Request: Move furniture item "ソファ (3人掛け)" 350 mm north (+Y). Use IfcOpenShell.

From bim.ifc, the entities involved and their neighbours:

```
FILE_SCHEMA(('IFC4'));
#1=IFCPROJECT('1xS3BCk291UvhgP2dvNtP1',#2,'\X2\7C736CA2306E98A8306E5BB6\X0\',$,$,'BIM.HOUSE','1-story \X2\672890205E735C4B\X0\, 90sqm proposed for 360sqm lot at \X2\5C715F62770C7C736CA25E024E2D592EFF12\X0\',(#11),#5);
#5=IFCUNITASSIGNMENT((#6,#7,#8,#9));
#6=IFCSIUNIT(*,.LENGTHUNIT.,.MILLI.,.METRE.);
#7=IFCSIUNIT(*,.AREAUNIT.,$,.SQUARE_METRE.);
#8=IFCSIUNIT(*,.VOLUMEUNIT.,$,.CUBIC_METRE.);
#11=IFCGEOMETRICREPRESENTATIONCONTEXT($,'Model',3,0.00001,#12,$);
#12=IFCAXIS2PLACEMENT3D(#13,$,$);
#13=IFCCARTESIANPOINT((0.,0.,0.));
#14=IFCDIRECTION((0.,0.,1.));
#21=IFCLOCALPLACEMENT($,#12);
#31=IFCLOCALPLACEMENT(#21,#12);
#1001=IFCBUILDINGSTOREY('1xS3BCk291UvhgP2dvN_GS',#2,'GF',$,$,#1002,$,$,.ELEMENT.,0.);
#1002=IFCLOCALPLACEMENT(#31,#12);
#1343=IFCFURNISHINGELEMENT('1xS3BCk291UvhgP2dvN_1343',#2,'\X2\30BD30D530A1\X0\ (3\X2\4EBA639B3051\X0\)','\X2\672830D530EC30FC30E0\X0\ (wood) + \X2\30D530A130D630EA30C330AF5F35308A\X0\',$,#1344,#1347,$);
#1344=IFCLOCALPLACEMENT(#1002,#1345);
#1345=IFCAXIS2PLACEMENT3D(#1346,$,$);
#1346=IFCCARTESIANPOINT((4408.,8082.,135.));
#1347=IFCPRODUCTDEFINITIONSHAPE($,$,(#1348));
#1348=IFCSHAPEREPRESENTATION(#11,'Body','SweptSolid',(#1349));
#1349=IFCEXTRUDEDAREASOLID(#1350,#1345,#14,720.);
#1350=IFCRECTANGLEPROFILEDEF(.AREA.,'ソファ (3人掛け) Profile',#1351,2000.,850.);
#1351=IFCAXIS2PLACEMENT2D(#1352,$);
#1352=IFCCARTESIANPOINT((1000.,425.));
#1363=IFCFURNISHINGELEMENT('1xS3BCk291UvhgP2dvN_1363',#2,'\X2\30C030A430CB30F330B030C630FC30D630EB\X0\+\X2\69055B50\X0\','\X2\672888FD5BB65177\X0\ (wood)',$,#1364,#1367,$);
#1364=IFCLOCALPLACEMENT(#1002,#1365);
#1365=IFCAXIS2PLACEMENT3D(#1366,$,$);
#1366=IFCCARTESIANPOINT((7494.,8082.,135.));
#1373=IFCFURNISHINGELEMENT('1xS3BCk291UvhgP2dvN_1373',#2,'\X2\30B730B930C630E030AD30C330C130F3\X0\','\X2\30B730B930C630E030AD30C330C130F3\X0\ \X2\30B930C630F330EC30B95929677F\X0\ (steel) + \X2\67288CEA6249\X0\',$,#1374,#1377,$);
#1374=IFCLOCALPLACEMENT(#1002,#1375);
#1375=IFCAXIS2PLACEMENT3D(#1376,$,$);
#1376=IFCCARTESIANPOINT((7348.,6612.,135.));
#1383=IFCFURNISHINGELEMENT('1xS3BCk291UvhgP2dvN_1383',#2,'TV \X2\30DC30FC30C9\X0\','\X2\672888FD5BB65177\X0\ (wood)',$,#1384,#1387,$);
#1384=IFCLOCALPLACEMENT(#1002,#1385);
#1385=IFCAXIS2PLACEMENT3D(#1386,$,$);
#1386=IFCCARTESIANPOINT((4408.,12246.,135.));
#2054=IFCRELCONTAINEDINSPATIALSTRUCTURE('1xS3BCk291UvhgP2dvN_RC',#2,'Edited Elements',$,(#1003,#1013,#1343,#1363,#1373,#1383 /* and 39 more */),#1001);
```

```python
import ifcopenshell
import ifcopenshell.api.geometry
import ifcopenshell.util.placement
import ifcopenshell.util.unit

model = ifcopenshell.open("bim.ifc")
unit_scale = ifcopenshell.util.unit.calculate_unit_scale(model)

item = model.by_guid("1xS3BCk291UvhgP2dvN_1343")
matrix = ifcopenshell.util.placement.get_local_placement(item.ObjectPlacement)
matrix[1, 3] += 0.35 / unit_scale
ifcopenshell.api.geometry.edit_object_placement(model, product=item, matrix=matrix, is_si=False)

print(ifcopenshell.util.placement.get_local_placement(item.ObjectPlacement).round(3) + 0.0)

model.write("bim_edited.ifc")
```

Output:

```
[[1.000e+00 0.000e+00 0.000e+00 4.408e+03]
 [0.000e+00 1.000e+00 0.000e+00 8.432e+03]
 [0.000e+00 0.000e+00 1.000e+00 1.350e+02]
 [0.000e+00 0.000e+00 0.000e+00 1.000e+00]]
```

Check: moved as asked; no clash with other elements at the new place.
